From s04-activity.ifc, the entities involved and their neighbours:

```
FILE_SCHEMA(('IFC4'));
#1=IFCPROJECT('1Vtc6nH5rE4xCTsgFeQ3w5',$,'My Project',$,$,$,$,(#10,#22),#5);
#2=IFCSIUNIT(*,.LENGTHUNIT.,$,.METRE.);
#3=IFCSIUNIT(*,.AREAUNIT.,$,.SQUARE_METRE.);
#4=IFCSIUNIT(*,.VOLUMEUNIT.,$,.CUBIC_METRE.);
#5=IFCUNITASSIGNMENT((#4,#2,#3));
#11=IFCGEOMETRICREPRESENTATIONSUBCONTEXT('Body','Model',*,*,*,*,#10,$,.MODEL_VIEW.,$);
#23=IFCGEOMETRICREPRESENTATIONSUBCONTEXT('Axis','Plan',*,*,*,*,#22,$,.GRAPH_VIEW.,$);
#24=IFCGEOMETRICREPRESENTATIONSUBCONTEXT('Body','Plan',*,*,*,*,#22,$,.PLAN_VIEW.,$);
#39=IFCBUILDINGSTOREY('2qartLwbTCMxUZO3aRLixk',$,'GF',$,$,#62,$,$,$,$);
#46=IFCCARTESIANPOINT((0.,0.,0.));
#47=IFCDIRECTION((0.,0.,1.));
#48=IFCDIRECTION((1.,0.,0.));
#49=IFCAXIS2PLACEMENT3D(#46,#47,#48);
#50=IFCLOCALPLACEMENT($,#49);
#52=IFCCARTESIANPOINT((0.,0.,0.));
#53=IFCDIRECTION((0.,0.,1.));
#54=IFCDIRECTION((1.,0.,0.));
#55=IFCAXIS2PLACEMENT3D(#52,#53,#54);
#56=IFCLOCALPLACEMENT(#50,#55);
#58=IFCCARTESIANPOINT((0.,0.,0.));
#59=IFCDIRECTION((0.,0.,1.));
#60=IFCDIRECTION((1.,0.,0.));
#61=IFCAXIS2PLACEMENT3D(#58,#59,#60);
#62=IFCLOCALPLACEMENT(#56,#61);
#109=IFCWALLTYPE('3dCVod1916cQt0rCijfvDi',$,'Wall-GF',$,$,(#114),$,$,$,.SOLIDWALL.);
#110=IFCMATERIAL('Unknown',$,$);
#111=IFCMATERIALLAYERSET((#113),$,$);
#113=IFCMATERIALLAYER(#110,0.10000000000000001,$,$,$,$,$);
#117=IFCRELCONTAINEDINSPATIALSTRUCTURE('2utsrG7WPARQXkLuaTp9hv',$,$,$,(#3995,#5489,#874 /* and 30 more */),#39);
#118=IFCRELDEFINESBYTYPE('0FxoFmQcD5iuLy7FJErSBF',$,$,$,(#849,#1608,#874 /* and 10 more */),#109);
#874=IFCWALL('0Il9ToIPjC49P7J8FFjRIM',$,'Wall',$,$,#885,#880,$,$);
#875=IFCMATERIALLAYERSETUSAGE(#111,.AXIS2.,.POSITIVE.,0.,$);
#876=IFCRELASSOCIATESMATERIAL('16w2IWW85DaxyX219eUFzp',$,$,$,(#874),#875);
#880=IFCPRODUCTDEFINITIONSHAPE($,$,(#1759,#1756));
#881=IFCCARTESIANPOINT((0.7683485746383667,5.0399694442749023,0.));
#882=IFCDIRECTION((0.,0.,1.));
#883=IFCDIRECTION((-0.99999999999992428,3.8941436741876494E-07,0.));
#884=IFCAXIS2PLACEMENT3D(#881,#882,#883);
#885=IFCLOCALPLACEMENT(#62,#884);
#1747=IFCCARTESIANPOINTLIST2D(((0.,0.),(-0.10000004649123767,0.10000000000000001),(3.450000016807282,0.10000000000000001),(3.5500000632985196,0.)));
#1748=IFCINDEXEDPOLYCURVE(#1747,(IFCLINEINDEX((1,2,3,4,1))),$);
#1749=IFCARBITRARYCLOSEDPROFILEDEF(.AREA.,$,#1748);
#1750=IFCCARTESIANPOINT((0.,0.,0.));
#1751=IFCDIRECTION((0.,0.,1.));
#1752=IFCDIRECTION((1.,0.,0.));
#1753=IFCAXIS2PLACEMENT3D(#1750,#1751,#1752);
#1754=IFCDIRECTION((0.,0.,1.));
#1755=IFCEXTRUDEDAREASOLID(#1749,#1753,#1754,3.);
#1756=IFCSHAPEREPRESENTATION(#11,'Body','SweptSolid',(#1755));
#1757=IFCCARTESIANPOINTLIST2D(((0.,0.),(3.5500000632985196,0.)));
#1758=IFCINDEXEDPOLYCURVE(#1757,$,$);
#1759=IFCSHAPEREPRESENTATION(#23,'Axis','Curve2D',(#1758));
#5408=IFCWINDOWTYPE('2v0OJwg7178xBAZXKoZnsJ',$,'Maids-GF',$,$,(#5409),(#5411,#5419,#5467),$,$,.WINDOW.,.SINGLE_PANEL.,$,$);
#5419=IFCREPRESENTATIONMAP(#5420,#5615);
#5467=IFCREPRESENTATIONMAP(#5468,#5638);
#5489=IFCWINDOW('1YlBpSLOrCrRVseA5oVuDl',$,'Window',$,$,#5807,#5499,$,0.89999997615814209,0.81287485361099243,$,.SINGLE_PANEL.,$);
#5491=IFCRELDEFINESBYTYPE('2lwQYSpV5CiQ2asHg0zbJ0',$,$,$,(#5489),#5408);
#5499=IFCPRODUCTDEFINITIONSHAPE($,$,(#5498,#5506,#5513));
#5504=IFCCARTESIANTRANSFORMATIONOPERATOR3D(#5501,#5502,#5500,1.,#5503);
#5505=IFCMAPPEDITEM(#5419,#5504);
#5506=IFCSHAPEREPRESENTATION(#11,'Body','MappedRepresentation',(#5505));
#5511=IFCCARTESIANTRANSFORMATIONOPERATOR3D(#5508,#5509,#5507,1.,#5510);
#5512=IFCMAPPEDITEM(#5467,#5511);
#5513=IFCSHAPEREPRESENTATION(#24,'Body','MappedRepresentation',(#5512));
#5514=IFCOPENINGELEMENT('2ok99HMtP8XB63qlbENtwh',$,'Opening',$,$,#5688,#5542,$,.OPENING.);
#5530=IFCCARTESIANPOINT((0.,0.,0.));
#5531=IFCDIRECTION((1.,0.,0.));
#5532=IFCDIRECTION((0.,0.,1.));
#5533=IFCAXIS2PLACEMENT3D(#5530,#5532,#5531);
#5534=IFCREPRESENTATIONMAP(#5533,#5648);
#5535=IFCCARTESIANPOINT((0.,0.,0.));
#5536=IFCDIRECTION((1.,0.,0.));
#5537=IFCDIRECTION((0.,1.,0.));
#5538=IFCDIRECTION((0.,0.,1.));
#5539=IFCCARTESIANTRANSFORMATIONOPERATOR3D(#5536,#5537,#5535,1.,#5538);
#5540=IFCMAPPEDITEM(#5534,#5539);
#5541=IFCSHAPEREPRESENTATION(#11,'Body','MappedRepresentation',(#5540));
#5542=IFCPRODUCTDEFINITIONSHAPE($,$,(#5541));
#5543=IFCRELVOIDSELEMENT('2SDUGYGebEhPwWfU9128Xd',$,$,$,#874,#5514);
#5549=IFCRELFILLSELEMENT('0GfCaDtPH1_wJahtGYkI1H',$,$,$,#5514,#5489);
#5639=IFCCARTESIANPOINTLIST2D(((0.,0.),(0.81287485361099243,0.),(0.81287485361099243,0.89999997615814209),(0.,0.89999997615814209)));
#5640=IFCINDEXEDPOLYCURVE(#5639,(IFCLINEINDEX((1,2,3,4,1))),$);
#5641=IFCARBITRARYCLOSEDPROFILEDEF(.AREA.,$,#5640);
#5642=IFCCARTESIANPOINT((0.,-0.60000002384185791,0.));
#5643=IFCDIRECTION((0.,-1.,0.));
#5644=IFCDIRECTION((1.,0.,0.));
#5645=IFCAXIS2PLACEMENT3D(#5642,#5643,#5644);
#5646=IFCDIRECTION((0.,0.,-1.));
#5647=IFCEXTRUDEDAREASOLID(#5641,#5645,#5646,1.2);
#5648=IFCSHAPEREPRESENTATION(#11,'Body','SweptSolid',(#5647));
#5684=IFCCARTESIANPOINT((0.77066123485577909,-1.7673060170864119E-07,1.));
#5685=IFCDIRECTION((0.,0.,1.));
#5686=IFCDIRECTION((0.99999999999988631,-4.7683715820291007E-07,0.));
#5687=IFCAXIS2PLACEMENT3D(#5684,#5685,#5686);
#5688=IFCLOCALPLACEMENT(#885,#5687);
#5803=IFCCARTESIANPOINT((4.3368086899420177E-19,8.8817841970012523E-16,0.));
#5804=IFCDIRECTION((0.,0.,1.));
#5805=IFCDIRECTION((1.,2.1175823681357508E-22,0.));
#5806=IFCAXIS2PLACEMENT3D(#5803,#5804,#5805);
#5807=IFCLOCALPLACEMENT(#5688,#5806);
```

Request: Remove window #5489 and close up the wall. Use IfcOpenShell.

```python
import ifcopenshell
import ifcopenshell.api.feature
import ifcopenshell.api.root
import ifcopenshell.geom
import ifcopenshell.util.shape

model = ifcopenshell.open("s04-activity.ifc")
settings = ifcopenshell.geom.settings()


def volume(element):
    """Net volume in cubic metres, openings subtracted."""
    shape = ifcopenshell.geom.create_shape(settings, element)
    return ifcopenshell.util.shape.get_volume(shape.geometry)


window = model.by_guid("1YlBpSLOrCrRVseA5oVuDl")
opening = window.FillsVoids[0].RelatingOpeningElement
wall = opening.VoidsElements[0].RelatingBuildingElement
before = volume(wall)

ifcopenshell.api.root.remove_product(model, product=window)
ifcopenshell.api.feature.remove_feature(model, feature=opening)

after = volume(wall)

print(f"wall volume {before:.3f} -> {after:.3f} m3")

model.write("s04-activity_edited.ifc")
```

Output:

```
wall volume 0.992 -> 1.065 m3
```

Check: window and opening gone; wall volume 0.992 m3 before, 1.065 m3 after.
